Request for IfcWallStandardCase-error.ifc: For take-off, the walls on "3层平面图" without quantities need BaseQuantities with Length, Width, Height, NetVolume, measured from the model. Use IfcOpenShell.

First a look at what the model holds.

```python
import ifcopenshell
import ifcopenshell.util.element
import ifcopenshell.util.unit

model = ifcopenshell.open("IfcWallStandardCase-error.ifc")
print(model.schema)
for unit_type in ("LENGTHUNIT", "AREAUNIT", "VOLUMEUNIT"):
    print(unit_type, ifcopenshell.util.unit.calculate_unit_scale(model, unit_type))
storey = next(s for s in model.by_type("IfcBuildingStorey") if s.Name == "3层平面图")
walls = [e for e in ifcopenshell.util.element.get_decomposition(storey) if e.is_a("IfcWall")]
for e in sorted(walls, key=lambda e: e.id()):
    print(e.id(), e.is_a(), e.Name, list(ifcopenshell.util.element.get_psets(e, qtos_only=True)), sep=" | ")
```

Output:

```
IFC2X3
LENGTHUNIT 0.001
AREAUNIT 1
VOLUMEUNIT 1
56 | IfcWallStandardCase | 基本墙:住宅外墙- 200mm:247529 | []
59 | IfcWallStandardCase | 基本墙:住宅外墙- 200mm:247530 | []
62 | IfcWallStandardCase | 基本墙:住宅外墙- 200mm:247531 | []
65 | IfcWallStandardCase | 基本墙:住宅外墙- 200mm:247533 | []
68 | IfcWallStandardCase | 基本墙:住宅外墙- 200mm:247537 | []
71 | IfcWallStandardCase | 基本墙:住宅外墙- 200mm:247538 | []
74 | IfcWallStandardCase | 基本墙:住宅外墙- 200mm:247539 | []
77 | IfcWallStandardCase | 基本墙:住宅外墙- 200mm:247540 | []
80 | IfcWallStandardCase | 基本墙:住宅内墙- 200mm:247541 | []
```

```python
import ifcopenshell
import ifcopenshell.api.pset
import ifcopenshell.geom
import ifcopenshell.util.element
import ifcopenshell.util.shape
import ifcopenshell.util.unit

model = ifcopenshell.open("IfcWallStandardCase-error.ifc")
unit_scale = ifcopenshell.util.unit.calculate_unit_scale(model)
volume_scale = ifcopenshell.util.unit.calculate_unit_scale(model, "VOLUMEUNIT")
settings = ifcopenshell.geom.settings()

storey = next(s for s in model.by_type("IfcBuildingStorey") if s.Name == "3层平面图")
walls = [e for e in ifcopenshell.util.element.get_decomposition(storey) if e.is_a("IfcWall")]

for e in sorted(walls, key=lambda e: e.id()):
    if ifcopenshell.util.element.get_psets(e, qtos_only=True, should_inherit=False):
        continue
    # Geometry comes back in metres, in the element's own axes.
    shape = ifcopenshell.geom.create_shape(settings, e)
    values = {
        "Length": ifcopenshell.util.shape.get_x(shape.geometry) / unit_scale,
        "Width": ifcopenshell.util.shape.get_y(shape.geometry) / unit_scale,
        "Height": ifcopenshell.util.shape.get_z(shape.geometry) / unit_scale,
        "NetVolume": ifcopenshell.util.shape.get_volume(shape.geometry) / volume_scale,
    }
    qto = ifcopenshell.api.pset.add_qto(model, product=e, name="BaseQuantities")
    ifcopenshell.api.pset.edit_qto(model, qto=qto, properties=values)
    print(e.id(), {k: round(v, 3) for k, v in values.items()})

model.write("IfcWallStandardCase-error_updated.ifc")
```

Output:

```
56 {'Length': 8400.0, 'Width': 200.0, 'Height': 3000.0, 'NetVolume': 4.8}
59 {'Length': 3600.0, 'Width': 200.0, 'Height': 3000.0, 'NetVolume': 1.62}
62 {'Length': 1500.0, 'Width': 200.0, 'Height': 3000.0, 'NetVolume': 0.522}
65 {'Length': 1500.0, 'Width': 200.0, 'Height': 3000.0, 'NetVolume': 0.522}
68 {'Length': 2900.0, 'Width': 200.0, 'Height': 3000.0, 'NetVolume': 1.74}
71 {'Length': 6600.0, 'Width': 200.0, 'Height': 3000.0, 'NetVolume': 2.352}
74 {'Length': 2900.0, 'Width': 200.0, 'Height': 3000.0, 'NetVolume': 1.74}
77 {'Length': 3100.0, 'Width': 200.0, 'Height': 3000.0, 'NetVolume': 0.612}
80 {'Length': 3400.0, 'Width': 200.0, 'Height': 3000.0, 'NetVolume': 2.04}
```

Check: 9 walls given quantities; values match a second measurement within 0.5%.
